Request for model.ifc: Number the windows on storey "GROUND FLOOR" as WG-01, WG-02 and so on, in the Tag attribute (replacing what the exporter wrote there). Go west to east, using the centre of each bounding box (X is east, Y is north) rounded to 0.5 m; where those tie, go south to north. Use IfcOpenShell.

First a look at what the model holds.

```python
import ifcopenshell
import ifcopenshell.util.element
import ifcopenshell.util.placement

model = ifcopenshell.open("model.ifc")
print(model.schema)
storey = next(s for s in model.by_type("IfcBuildingStorey") if s.Name == "GROUND FLOOR")
windows = [e for e in ifcopenshell.util.element.get_decomposition(storey) if e.is_a("IfcWindow")]
for e in sorted(windows, key=lambda e: e.id()):
    origin = ifcopenshell.util.placement.get_local_placement(e.ObjectPlacement)[:3, 3]
    print(e.id(), e.Tag, e.Name, origin.round(2) + 0.0, sep=" | ")
```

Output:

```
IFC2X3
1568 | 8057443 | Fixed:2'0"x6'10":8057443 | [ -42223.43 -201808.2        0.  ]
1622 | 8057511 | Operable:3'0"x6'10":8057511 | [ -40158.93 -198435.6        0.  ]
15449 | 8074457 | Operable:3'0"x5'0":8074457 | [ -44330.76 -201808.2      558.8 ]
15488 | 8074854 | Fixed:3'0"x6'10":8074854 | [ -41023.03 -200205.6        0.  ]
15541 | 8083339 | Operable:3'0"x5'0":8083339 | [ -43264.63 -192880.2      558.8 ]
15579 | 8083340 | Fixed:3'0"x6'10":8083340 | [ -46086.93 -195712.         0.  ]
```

```python
import ifcopenshell
import ifcopenshell.geom
import ifcopenshell.util.element
import ifcopenshell.util.shape

model = ifcopenshell.open("model.ifc")
settings = ifcopenshell.geom.settings()
settings.set("use-world-coords", True)


def centre(element):
    shape = ifcopenshell.geom.create_shape(settings, element)
    return ifcopenshell.util.shape.get_bbox_centroid(shape.geometry)


storey = next(s for s in model.by_type("IfcBuildingStorey") if s.Name == "GROUND FLOOR")
windows = [e for e in ifcopenshell.util.element.get_decomposition(storey) if e.is_a("IfcWindow")]

# Insertion points can sit at a corner or the storey origin, so sort by the geometry (in metres).
centres = {e: centre(e) for e in windows}
windows.sort(key=lambda e: (round(centres[e][0] / 0.5), centres[e][1]))

for i, e in enumerate(windows, start=1):
    number = f"WG-{i:02d}"
    e.Tag = number
    print(e.id(), number)

model.write("model-out.ifc")
```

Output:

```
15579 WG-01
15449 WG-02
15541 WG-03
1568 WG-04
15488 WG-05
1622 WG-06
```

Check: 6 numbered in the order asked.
